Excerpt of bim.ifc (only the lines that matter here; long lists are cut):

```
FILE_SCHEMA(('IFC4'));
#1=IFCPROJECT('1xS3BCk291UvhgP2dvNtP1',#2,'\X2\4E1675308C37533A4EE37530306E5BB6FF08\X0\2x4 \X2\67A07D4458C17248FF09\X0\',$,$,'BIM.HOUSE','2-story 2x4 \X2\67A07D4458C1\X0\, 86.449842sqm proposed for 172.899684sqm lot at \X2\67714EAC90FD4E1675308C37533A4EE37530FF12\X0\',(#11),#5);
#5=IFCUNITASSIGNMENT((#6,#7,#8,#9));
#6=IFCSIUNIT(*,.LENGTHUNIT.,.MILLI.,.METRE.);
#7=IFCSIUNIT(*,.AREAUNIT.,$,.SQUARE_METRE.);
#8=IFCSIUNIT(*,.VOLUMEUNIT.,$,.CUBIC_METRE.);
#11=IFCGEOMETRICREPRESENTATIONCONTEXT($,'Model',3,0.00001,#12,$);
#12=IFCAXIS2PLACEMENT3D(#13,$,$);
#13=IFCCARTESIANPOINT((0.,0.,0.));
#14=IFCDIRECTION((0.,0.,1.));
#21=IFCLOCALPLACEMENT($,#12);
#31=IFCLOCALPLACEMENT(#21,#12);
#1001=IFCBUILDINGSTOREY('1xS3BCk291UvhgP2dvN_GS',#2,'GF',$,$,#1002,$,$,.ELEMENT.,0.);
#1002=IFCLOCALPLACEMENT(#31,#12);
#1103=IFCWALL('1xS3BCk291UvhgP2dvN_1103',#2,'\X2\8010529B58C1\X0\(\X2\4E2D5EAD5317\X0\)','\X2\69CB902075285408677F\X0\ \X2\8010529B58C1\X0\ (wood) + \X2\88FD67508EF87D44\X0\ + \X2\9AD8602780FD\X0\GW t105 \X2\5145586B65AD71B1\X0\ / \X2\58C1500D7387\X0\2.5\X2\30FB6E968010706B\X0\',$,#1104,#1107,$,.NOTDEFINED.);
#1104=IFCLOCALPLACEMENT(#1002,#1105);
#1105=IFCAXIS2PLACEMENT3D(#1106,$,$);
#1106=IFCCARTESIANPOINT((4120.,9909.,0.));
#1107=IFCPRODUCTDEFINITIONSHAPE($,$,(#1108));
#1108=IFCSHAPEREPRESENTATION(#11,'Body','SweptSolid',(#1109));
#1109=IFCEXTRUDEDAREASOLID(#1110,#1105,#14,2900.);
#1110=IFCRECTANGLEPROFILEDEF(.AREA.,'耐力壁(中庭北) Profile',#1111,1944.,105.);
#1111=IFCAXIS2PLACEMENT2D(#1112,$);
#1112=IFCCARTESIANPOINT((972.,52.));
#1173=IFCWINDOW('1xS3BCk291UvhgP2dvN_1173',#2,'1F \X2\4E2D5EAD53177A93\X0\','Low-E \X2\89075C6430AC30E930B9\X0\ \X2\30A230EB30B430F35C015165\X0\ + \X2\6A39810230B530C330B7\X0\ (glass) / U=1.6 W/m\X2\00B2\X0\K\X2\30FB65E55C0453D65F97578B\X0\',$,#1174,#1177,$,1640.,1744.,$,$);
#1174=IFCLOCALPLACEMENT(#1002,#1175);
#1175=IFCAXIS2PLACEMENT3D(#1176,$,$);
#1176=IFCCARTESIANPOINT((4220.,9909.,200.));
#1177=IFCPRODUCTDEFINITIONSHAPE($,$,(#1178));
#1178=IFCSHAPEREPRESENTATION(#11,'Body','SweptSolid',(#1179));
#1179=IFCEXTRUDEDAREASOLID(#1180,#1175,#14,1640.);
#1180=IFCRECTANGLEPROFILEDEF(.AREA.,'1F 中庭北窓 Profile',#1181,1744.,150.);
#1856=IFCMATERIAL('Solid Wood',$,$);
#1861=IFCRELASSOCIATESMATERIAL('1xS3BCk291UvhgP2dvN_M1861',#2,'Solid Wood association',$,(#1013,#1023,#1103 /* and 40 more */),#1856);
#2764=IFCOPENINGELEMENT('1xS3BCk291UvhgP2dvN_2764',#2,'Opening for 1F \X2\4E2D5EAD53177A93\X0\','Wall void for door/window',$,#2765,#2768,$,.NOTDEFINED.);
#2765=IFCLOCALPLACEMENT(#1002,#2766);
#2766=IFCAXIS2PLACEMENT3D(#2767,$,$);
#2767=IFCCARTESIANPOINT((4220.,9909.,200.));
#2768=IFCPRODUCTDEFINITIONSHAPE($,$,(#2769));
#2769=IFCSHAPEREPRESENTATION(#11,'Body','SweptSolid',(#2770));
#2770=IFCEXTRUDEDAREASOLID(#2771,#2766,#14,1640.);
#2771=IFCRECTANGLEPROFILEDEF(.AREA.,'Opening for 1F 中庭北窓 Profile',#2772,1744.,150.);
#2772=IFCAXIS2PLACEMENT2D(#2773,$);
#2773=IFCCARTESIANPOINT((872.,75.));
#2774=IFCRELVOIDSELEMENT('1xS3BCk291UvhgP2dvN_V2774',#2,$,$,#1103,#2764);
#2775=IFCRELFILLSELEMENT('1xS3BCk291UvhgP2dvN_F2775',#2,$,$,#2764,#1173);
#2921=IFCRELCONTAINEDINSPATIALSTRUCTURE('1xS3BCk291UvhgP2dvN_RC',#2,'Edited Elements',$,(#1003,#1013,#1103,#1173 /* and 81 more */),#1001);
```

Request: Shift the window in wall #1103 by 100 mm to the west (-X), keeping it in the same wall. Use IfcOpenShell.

```python
import ifcopenshell
import ifcopenshell.api.geometry
import ifcopenshell.util.placement

model = ifcopenshell.open("bim.ifc")

window = model.by_id(1173)
opening = window.FillsVoids[0].RelatingOpeningElement
wall = opening.VoidsElements[0].RelatingBuildingElement

wall_matrix = ifcopenshell.util.placement.get_local_placement(wall.ObjectPlacement)
shift = wall_matrix[:3, 0] * -100.0
before = ifcopenshell.util.placement.get_local_placement(window.ObjectPlacement)[:3, 3].copy()

# The window is not placed relative to its opening, so move both.
for product in (opening, window):
    matrix = ifcopenshell.util.placement.get_local_placement(product.ObjectPlacement)
    matrix[:3, 3] += shift
    ifcopenshell.api.geometry.edit_object_placement(model, product=product, matrix=matrix, is_si=False)

after = ifcopenshell.util.placement.get_local_placement(window.ObjectPlacement)[:3, 3]
print("window moved by", (after - before).round(3) + 0.0)

model.write("bim-out.ifc")
```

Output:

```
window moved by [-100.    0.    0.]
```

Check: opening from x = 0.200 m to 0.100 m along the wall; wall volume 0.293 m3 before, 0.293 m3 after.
